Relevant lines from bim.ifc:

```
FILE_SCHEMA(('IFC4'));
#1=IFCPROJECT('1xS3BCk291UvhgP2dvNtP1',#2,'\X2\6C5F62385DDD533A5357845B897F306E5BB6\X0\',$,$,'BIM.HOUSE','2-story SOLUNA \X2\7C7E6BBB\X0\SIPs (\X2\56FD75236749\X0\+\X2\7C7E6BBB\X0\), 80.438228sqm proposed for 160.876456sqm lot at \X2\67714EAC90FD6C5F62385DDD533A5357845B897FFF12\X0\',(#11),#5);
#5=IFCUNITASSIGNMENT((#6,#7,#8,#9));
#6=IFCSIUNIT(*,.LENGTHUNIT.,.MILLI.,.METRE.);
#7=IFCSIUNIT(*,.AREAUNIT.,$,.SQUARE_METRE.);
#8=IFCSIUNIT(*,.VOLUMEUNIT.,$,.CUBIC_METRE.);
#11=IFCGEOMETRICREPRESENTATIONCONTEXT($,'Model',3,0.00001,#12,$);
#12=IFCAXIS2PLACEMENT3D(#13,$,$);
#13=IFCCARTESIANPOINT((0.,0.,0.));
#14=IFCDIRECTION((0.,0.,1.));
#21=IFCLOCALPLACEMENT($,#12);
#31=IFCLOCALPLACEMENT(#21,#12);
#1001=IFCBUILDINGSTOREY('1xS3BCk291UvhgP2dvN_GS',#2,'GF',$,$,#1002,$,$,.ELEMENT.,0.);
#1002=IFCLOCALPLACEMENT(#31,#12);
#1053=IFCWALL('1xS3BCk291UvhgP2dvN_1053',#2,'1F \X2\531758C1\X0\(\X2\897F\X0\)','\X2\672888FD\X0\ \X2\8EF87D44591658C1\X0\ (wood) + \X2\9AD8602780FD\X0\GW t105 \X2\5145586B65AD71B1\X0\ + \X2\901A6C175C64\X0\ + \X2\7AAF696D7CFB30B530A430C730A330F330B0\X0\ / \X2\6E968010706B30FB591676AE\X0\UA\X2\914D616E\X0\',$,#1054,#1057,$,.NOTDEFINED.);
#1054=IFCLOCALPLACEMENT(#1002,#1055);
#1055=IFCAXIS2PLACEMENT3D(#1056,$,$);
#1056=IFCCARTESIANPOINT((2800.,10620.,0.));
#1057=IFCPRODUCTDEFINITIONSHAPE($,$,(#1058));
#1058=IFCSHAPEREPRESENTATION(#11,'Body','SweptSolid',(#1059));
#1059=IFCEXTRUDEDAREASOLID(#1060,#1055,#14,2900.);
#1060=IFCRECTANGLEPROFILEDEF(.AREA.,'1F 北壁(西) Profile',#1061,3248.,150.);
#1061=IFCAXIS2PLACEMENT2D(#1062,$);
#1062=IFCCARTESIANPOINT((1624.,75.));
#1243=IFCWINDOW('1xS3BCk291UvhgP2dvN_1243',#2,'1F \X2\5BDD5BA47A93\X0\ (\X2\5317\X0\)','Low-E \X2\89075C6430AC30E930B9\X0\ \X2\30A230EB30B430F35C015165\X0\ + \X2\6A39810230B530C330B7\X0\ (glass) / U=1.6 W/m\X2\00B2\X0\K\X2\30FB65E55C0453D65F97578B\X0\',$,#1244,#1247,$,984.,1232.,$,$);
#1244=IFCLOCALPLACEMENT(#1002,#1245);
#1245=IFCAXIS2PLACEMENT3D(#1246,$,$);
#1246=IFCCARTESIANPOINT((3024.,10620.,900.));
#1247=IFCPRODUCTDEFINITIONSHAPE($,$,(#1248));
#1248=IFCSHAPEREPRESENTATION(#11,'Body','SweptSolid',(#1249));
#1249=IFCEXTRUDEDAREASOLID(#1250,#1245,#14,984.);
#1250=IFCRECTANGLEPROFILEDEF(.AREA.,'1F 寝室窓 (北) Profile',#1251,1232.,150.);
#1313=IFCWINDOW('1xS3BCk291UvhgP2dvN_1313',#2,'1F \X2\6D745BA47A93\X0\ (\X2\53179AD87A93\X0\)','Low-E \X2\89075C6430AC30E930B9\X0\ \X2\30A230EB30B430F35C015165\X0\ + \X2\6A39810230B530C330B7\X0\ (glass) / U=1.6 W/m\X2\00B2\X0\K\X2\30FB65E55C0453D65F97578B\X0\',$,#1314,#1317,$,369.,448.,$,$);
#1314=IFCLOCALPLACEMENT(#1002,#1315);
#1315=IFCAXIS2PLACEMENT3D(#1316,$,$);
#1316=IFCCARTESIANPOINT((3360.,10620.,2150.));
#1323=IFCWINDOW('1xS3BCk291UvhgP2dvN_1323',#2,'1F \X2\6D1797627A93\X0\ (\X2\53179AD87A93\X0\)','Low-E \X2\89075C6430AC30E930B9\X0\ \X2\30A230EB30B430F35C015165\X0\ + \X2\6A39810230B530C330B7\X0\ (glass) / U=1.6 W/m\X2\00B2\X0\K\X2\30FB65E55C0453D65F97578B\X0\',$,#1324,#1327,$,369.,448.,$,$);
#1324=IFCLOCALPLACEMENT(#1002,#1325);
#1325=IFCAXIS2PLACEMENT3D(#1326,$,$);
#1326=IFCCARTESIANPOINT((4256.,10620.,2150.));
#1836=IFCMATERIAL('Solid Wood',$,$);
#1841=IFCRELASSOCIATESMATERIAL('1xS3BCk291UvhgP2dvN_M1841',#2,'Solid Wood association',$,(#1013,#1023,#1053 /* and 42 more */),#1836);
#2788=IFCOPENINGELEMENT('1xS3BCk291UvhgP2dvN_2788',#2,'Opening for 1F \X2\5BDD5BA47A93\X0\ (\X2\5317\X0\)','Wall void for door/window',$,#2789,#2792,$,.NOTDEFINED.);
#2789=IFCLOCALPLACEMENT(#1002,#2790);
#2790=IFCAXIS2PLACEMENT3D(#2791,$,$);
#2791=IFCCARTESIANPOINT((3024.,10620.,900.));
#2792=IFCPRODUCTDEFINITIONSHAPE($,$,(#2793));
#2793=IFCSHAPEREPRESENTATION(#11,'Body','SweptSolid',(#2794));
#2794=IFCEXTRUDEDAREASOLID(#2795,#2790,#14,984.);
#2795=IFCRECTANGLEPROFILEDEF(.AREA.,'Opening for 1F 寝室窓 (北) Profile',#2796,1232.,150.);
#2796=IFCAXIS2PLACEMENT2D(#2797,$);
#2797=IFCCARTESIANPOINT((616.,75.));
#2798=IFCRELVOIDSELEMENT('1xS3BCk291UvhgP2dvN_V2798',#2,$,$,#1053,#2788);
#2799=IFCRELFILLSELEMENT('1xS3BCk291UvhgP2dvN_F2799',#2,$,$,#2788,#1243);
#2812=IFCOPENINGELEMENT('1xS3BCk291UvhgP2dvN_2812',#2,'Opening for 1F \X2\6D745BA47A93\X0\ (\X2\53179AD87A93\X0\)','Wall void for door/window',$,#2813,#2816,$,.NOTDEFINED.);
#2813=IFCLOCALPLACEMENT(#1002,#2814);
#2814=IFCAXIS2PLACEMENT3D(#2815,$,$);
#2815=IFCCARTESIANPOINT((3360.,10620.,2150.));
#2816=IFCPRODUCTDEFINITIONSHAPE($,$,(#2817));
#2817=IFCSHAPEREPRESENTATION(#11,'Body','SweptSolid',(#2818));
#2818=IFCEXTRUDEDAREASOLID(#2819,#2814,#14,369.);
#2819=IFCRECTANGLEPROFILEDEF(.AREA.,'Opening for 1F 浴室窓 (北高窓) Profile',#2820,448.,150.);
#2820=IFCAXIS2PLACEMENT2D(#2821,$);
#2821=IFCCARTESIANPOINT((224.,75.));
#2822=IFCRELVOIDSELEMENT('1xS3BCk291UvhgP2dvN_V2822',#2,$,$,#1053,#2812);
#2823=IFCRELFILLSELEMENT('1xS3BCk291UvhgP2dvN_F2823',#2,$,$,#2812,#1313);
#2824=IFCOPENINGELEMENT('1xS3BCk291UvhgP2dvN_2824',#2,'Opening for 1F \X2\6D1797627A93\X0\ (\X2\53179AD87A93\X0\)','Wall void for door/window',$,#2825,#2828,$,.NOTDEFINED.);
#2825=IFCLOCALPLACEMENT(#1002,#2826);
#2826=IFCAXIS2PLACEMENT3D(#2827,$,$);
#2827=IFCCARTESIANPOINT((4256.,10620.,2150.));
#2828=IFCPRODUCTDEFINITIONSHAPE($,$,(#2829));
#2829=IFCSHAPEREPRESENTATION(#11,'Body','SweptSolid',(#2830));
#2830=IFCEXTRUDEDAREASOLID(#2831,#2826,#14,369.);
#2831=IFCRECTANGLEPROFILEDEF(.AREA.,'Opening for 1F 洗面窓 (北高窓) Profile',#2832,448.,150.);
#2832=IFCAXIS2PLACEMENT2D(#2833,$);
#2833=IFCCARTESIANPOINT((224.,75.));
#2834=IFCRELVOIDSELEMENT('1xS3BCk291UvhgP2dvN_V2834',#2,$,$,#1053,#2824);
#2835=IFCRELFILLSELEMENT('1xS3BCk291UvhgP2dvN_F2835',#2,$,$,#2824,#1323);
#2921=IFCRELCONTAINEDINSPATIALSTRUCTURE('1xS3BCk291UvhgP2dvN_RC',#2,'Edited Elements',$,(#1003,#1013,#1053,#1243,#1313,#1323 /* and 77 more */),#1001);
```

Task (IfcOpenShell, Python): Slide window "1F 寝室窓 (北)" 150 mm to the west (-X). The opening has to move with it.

```python
import ifcopenshell
import ifcopenshell.api.geometry
import ifcopenshell.util.placement

model = ifcopenshell.open("bim.ifc")

window = model.by_id(1243)
opening = window.FillsVoids[0].RelatingOpeningElement
wall = opening.VoidsElements[0].RelatingBuildingElement

wall_matrix = ifcopenshell.util.placement.get_local_placement(wall.ObjectPlacement)
shift = wall_matrix[:3, 0] * -150.0
before = ifcopenshell.util.placement.get_local_placement(window.ObjectPlacement)[:3, 3].copy()

# The window is not placed relative to its opening, so move both.
for product in (opening, window):
    matrix = ifcopenshell.util.placement.get_local_placement(product.ObjectPlacement)
    matrix[:3, 3] += shift
    ifcopenshell.api.geometry.edit_object_placement(model, product=product, matrix=matrix, is_si=False)

after = ifcopenshell.util.placement.get_local_placement(window.ObjectPlacement)[:3, 3]
print("window moved by", (after - before).round(3) + 0.0)

model.write("bim-out.ifc")
```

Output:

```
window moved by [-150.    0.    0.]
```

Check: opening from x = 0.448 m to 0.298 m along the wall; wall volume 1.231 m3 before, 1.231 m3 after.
